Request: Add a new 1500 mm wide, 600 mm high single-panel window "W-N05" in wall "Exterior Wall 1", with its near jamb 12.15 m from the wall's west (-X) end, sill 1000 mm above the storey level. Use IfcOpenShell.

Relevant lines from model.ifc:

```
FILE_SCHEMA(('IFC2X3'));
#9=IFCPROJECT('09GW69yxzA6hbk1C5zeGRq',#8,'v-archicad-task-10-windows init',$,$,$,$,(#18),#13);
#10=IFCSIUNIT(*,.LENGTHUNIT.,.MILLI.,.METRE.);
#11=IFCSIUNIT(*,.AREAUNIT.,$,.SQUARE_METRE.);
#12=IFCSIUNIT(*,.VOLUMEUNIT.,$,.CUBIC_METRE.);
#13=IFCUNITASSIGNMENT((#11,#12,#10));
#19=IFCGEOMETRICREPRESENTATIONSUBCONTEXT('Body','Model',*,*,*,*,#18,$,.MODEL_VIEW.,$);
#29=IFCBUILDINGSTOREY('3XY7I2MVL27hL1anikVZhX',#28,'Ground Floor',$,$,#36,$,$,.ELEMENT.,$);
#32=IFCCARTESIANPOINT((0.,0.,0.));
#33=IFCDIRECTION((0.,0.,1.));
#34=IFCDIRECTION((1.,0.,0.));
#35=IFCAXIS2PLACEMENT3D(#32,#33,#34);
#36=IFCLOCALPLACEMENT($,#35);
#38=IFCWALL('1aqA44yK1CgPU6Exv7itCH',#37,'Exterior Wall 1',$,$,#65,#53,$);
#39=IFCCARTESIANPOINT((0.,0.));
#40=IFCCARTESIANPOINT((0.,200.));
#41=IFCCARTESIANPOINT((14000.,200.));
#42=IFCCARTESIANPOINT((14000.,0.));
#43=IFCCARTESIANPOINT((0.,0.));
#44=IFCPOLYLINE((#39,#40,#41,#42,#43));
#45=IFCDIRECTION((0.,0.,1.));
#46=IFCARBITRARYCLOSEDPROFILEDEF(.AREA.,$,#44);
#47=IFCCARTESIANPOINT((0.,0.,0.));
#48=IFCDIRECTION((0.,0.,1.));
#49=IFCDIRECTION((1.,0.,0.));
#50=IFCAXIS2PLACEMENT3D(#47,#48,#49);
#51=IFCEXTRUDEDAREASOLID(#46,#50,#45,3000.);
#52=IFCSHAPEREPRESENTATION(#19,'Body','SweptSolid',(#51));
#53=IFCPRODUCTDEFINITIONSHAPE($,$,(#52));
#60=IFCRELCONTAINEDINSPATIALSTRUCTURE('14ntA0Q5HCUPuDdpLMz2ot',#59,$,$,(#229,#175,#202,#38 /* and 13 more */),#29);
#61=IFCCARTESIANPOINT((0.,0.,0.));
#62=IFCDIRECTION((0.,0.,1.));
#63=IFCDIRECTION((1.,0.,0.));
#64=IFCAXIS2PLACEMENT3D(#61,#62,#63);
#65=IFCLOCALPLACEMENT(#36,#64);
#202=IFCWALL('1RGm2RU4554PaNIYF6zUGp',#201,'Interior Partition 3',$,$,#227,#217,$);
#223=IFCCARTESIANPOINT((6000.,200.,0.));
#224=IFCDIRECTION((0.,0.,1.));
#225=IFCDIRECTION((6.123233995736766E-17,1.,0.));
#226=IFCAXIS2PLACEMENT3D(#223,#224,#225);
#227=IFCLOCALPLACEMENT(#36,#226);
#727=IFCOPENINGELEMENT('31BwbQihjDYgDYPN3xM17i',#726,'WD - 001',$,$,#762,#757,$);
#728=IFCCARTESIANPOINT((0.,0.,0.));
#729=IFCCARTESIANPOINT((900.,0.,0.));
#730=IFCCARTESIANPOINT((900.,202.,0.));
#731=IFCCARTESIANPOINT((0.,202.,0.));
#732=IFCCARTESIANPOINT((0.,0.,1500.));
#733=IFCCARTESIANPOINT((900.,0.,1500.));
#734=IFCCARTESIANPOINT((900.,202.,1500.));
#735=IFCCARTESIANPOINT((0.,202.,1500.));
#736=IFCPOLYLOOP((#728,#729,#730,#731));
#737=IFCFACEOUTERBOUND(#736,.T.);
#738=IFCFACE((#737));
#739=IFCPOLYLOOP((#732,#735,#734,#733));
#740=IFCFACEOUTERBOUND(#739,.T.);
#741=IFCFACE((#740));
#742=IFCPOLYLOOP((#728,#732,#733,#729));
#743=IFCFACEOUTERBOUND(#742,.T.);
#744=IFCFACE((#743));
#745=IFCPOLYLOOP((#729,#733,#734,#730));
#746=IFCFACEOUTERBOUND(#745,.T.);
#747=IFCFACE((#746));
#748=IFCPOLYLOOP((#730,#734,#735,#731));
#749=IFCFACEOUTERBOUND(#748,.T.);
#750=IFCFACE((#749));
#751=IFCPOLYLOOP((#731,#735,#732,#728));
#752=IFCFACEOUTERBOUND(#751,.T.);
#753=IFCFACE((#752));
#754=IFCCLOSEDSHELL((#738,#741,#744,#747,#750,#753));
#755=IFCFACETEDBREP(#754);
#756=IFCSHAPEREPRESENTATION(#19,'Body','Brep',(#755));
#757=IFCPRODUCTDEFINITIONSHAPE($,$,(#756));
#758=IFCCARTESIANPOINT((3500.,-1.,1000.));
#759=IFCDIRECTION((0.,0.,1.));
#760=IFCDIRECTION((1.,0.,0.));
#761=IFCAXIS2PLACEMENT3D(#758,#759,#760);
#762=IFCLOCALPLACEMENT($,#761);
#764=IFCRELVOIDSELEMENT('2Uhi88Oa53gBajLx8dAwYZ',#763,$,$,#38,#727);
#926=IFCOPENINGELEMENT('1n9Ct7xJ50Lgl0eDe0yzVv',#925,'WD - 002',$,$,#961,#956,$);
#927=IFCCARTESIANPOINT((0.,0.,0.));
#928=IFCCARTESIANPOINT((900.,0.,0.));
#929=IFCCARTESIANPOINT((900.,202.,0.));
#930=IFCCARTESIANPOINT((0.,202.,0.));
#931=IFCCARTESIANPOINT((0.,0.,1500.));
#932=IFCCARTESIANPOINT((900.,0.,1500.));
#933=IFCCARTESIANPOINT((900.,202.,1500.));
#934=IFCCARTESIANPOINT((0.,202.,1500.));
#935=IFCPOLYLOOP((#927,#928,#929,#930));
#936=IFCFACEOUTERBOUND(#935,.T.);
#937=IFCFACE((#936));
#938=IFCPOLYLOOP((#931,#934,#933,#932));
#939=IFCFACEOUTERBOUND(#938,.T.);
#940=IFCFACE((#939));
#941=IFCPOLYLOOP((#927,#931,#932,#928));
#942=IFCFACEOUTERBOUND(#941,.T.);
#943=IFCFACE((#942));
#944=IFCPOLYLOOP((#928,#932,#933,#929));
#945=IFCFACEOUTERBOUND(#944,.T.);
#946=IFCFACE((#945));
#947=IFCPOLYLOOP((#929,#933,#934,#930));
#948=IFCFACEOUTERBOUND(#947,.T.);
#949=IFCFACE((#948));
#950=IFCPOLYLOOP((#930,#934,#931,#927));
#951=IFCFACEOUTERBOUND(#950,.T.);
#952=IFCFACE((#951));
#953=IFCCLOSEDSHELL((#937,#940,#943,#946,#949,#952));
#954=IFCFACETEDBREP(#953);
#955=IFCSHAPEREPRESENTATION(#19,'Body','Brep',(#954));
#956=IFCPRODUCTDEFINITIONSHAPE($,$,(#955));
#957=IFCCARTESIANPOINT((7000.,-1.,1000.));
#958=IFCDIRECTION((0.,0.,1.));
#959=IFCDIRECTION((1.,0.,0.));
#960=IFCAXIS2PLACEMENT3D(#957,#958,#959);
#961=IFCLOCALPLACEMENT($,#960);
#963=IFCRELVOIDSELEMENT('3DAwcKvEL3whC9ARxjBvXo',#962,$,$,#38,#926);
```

```python
import numpy as np
import ifcopenshell
import ifcopenshell.api.feature
import ifcopenshell.api.geometry
import ifcopenshell.api.root
import ifcopenshell.api.spatial
import ifcopenshell.api.type
import ifcopenshell.geom
import ifcopenshell.util.element
import ifcopenshell.util.placement
import ifcopenshell.util.representation
import ifcopenshell.util.shape
import ifcopenshell.util.unit

model = ifcopenshell.open("model.ifc")
unit_scale = ifcopenshell.util.unit.calculate_unit_scale(model)
settings = ifcopenshell.geom.settings()


def volume(element):
    """Net volume in cubic metres, openings subtracted."""
    shape = ifcopenshell.geom.create_shape(settings, element)
    return ifcopenshell.util.shape.get_volume(shape.geometry)


wall = model.by_id(38)
storey = ifcopenshell.util.element.get_container(wall, ifc_class="IfcBuildingStorey")
context = ifcopenshell.util.representation.get_context(model, "Model", "Body", "MODEL_VIEW")
before = volume(wall)

width, height, from_end, sill = 1.5, 0.6, 12.15, 1  # metres

# The wall runs along its own X axis, and the end named is its -X end.
wall_shape = ifcopenshell.geom.create_shape(settings, wall)
x, y, z = ifcopenshell.util.shape.get_vertices(wall_shape.geometry).T
start = x.min() + from_end
face, thickness = float(y.min()), float(y.max() - y.min())
wall_matrix = ifcopenshell.util.placement.get_local_placement(wall.ObjectPlacement)
level = ifcopenshell.util.placement.get_local_placement(storey.ObjectPlacement)[2, 3]


def in_wall(x, y):
    """Placement at x, y metres in the wall's axes, at sill height."""
    matrix = wall_matrix.copy()
    matrix[:, 3] = wall_matrix @ np.array([x / unit_scale, y / unit_scale, 0.0, 1.0])
    matrix[2, 3] = level + sill / unit_scale
    return matrix


# Opening: a box that overshoots both wall faces by 50 mm.
opening = ifcopenshell.api.root.create_entity(model, ifc_class="IfcOpeningElement")
box = ifcopenshell.api.geometry.add_wall_representation(
    model, context=context, length=width, height=height, thickness=thickness + 0.1
)
ifcopenshell.api.geometry.assign_representation(model, product=opening, representation=box)
ifcopenshell.api.geometry.edit_object_placement(model, product=opening, matrix=in_wall(start, face - 0.05), is_si=False)
ifcopenshell.api.feature.add_feature(model, feature=opening, element=wall)

window = ifcopenshell.api.root.create_entity(model, ifc_class="IfcWindow", name="W-N05")
window.OverallWidth, window.OverallHeight = width / unit_scale, height / unit_scale
body = ifcopenshell.api.geometry.add_window_representation(
    model,
    context=context,
    overall_width=window.OverallWidth,
    overall_height=window.OverallHeight,
    partition_type="SINGLE_PANEL",
)
ifcopenshell.api.geometry.assign_representation(model, product=window, representation=body)
ifcopenshell.api.spatial.assign_container(model, products=[window], relating_structure=storey)
fills = ifcopenshell.api.feature.add_filling(model, opening=opening, element=window)
fills.OwnerHistory = window.OwnerHistory  # required in IFC2X3

# IFC2X3 keeps the operation on the window style.
style = ifcopenshell.api.root.create_entity(model, ifc_class="IfcWindowStyle", name="W-N05")
style.OperationType, style.ConstructionType = "SINGLE_PANEL", "NOTDEFINED"
style.ParameterTakesPrecedence = style.Sizeable = False
ifcopenshell.api.type.assign_type(model, related_objects=[window], relating_type=style)

# Centre the window in the wall's thickness.
ifcopenshell.api.geometry.edit_object_placement(model, product=window, matrix=in_wall(start, face), is_si=False)
window_shape = ifcopenshell.geom.create_shape(settings, window)
depth = ifcopenshell.util.shape.get_vertices(window_shape.geometry)[:, 1]
offset = face + thickness / 2 - (depth.min() + depth.max()) / 2
ifcopenshell.api.geometry.edit_object_placement(model, product=window, matrix=in_wall(start, offset), is_si=False)

after = volume(wall)

print(f"wall volume {before:.3f} -> {after:.3f} m3")

model.write("model_updated.ifc")
```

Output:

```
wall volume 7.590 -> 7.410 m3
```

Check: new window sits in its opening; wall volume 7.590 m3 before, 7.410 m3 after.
